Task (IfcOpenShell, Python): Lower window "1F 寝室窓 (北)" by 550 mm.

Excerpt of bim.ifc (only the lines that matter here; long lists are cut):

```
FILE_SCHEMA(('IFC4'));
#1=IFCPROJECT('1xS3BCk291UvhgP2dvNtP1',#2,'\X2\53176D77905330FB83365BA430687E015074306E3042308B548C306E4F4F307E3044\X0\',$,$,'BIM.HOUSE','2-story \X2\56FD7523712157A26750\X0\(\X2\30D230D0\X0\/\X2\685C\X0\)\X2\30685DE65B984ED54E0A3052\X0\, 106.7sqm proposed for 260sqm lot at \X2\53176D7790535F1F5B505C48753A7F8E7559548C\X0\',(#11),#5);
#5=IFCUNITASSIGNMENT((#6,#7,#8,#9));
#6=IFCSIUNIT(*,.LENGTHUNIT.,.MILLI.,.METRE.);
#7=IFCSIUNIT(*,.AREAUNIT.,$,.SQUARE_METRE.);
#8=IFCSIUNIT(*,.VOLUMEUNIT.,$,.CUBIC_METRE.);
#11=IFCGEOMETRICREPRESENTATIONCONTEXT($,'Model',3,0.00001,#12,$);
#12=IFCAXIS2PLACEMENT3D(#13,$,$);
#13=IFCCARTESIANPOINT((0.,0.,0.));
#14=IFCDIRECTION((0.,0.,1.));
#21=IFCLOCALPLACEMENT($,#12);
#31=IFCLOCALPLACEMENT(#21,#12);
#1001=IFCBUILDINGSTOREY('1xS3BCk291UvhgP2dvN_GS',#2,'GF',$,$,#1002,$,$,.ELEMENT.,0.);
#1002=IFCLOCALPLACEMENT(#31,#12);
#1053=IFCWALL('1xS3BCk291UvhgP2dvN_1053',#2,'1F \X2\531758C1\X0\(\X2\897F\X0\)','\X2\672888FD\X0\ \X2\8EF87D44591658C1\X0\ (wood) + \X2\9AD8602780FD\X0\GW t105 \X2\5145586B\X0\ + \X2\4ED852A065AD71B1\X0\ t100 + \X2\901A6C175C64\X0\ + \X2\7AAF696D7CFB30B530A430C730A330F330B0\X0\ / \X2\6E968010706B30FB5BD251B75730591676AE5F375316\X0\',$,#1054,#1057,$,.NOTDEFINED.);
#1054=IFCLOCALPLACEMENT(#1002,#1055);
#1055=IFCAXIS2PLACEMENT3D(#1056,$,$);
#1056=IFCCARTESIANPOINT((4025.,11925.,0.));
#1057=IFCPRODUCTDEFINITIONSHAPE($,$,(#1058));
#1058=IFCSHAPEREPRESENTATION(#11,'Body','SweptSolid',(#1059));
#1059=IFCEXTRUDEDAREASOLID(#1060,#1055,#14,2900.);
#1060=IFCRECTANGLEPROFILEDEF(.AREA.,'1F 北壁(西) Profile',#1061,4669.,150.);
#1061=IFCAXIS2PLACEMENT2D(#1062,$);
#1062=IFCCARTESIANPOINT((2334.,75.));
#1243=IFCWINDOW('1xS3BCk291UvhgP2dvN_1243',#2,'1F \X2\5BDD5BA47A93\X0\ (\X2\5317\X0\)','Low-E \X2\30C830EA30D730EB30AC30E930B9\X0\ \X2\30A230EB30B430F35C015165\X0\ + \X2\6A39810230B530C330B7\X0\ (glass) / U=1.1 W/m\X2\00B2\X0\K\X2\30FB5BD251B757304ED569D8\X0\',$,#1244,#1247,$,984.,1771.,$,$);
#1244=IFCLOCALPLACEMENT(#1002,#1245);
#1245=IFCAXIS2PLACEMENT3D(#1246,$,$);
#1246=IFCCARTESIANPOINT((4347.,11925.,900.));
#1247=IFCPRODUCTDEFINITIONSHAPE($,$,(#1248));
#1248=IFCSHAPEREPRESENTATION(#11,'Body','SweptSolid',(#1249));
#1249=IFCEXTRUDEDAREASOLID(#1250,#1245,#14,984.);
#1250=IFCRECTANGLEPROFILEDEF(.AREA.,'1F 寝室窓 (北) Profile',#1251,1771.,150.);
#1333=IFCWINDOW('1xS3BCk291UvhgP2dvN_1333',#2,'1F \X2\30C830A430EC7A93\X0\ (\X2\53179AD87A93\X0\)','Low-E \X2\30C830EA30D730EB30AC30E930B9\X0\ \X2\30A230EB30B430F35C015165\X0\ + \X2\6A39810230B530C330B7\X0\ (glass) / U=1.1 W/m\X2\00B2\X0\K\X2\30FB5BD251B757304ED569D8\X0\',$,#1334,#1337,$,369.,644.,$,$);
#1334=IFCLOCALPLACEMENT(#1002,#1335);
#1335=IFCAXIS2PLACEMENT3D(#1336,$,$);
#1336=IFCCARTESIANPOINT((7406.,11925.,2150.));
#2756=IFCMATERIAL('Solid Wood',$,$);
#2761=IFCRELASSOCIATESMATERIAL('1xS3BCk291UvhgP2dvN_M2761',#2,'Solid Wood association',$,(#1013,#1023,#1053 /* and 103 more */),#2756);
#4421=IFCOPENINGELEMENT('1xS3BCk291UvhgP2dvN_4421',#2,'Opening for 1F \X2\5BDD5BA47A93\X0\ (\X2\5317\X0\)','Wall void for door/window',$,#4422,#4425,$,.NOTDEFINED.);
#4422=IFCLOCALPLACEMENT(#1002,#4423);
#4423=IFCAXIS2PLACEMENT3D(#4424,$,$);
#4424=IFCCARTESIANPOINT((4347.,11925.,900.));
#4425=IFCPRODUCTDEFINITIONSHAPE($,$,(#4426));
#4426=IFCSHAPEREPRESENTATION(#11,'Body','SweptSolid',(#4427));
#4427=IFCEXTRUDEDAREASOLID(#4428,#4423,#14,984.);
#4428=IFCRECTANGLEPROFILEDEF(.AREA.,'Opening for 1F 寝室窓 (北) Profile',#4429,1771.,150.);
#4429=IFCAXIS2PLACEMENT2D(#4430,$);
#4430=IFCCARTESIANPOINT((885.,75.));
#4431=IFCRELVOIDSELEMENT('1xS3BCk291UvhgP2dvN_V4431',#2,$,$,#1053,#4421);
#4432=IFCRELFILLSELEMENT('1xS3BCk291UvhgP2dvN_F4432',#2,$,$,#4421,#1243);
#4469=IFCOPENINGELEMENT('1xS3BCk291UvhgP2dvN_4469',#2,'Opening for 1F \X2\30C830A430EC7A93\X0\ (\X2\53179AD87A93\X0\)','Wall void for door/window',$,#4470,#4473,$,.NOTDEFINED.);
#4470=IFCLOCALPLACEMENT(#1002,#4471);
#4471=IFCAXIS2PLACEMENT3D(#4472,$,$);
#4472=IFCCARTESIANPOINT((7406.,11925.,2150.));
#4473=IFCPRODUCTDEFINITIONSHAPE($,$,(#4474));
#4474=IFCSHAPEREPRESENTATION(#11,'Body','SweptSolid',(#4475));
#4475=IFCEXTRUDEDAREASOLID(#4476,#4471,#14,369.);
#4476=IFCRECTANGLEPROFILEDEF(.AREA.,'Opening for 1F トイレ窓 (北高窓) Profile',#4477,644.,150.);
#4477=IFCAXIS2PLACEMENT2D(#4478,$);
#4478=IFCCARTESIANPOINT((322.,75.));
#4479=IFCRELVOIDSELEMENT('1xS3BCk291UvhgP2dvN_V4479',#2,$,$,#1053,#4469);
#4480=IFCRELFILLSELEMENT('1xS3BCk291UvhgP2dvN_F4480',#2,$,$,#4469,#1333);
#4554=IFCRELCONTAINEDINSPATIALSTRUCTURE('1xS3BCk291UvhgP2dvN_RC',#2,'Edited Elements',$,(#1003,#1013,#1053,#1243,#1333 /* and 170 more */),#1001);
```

```python
import numpy as np
import ifcopenshell
import ifcopenshell.api.geometry
import ifcopenshell.util.placement
import ifcopenshell.util.unit

model = ifcopenshell.open("bim.ifc")
unit_scale = ifcopenshell.util.unit.calculate_unit_scale(model)

window = model.by_guid("1xS3BCk291UvhgP2dvN_1243")
opening = window.FillsVoids[0].RelatingOpeningElement
dz = -0.55 / unit_scale

shift = np.array([0.0, 0.0, dz])
# The window is not placed relative to its opening, so move both.
for product in (opening, window):
    matrix = ifcopenshell.util.placement.get_local_placement(product.ObjectPlacement)
    matrix[:3, 3] += shift
    ifcopenshell.api.geometry.edit_object_placement(model, product=product, matrix=matrix, is_si=False)

print(f"moved by {dz * unit_scale:+.3f} m")

model.write("bim_edited.ifc")
```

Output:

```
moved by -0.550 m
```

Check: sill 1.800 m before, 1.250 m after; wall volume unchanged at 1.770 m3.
